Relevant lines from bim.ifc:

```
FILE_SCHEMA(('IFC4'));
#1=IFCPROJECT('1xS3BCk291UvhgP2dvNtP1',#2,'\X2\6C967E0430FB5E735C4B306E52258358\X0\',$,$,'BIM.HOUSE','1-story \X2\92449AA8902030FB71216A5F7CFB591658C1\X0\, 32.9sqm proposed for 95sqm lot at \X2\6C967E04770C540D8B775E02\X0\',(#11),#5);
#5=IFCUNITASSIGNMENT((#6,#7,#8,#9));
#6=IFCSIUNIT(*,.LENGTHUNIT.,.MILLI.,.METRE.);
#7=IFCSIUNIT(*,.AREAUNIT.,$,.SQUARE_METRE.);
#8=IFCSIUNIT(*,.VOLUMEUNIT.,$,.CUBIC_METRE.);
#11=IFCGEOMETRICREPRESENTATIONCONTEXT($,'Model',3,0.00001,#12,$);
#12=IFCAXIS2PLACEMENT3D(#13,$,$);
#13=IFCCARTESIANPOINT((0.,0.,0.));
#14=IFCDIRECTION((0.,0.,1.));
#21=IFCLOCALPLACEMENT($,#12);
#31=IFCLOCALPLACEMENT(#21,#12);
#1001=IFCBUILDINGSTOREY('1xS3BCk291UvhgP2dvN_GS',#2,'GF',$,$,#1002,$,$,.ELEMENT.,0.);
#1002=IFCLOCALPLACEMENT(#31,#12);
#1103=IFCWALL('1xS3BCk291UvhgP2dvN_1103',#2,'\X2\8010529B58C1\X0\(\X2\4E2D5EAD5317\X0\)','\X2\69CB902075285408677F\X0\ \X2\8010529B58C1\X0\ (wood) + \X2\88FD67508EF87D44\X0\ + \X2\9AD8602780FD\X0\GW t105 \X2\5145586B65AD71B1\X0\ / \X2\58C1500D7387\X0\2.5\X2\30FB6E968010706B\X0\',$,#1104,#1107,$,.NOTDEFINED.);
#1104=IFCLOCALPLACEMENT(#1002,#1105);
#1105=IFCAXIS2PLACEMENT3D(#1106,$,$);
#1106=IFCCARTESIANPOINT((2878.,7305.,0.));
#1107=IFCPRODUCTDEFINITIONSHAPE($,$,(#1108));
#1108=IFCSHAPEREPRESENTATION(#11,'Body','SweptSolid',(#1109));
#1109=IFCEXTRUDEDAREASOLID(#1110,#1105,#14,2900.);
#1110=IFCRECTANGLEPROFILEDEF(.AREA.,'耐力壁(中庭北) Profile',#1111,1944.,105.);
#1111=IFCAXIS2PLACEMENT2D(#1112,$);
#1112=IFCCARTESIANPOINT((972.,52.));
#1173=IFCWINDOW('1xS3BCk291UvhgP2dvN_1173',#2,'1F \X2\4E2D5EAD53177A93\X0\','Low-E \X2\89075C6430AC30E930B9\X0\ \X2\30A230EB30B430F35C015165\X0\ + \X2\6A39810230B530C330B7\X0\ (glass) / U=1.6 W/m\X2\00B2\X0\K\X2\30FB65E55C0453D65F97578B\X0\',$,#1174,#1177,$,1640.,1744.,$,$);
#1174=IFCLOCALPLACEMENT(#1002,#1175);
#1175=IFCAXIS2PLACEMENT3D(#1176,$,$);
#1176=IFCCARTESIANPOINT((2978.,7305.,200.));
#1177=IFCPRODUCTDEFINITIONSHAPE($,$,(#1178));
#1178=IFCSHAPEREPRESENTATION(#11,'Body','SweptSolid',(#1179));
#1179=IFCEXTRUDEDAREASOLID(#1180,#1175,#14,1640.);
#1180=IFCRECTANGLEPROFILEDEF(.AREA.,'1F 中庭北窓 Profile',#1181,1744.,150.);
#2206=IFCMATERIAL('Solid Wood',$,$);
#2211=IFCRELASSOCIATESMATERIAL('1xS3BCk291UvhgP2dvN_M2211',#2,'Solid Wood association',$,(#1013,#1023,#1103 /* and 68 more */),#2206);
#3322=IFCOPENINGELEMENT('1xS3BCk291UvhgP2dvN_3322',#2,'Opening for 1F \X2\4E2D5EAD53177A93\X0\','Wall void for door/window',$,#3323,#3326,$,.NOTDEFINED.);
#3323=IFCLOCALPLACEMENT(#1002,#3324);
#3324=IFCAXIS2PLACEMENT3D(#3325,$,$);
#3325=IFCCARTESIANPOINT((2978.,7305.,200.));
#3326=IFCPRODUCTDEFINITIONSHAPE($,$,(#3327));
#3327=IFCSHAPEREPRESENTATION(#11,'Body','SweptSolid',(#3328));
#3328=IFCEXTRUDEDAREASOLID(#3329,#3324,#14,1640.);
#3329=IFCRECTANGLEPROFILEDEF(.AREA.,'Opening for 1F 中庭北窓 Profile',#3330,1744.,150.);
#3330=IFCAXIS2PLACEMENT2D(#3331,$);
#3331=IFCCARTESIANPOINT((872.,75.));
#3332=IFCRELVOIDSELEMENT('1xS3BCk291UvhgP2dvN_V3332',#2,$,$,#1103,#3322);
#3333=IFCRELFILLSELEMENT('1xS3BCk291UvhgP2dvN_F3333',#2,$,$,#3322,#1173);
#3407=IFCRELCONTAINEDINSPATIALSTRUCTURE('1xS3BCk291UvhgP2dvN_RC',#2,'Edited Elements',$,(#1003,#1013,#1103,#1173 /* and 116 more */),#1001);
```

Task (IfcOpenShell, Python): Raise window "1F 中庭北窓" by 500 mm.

```python
import numpy as np
import ifcopenshell
import ifcopenshell.api.geometry
import ifcopenshell.util.placement
import ifcopenshell.util.unit

model = ifcopenshell.open("bim.ifc")
unit_scale = ifcopenshell.util.unit.calculate_unit_scale(model)

window = model.by_guid("1xS3BCk291UvhgP2dvN_1173")
opening = window.FillsVoids[0].RelatingOpeningElement
dz = 500.0

shift = np.array([0.0, 0.0, dz])
# The window is not placed relative to its opening, so move both.
for product in (opening, window):
    matrix = ifcopenshell.util.placement.get_local_placement(product.ObjectPlacement)
    matrix[:3, 3] += shift
    ifcopenshell.api.geometry.edit_object_placement(model, product=product, matrix=matrix, is_si=False)

print(f"moved by {dz * unit_scale:+.3f} m")

model.write("bim_v2.ifc")
```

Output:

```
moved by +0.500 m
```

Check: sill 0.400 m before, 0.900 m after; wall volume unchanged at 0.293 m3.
